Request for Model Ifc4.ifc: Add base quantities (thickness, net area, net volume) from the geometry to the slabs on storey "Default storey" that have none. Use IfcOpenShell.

First a look at what the model holds.

```python
import ifcopenshell
import ifcopenshell.util.element
import ifcopenshell.util.unit

model = ifcopenshell.open("Model Ifc4.ifc")
print(model.schema)
for unit_type in ("LENGTHUNIT", "AREAUNIT", "VOLUMEUNIT"):
    print(unit_type, ifcopenshell.util.unit.calculate_unit_scale(model, unit_type))
storey = next(s for s in model.by_type("IfcBuildingStorey") if s.Name == "Default storey")
slabs = [e for e in ifcopenshell.util.element.get_decomposition(storey) if e.is_a("IfcSlab")]
for e in sorted(slabs, key=lambda e: e.id()):
    print(e.id(), e.is_a(), e.Name, list(ifcopenshell.util.element.get_psets(e, qtos_only=True)), sep=" | ")
```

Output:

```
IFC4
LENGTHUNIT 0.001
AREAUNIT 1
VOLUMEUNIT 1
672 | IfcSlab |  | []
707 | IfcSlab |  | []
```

```python
import ifcopenshell
import ifcopenshell.api.pset
import ifcopenshell.geom
import ifcopenshell.util.element
import ifcopenshell.util.shape
import ifcopenshell.util.unit

model = ifcopenshell.open("Model Ifc4.ifc")
unit_scale = ifcopenshell.util.unit.calculate_unit_scale(model)
area_scale = ifcopenshell.util.unit.calculate_unit_scale(model, "AREAUNIT")
volume_scale = ifcopenshell.util.unit.calculate_unit_scale(model, "VOLUMEUNIT")
settings = ifcopenshell.geom.settings()

storey = next(s for s in model.by_type("IfcBuildingStorey") if s.Name == "Default storey")
slabs = [e for e in ifcopenshell.util.element.get_decomposition(storey) if e.is_a("IfcSlab")]

for e in sorted(slabs, key=lambda e: e.id()):
    if ifcopenshell.util.element.get_psets(e, qtos_only=True, should_inherit=False):
        continue
    # Geometry comes back in metres, in the element's own axes.
    shape = ifcopenshell.geom.create_shape(settings, e)
    values = {
        "Width": ifcopenshell.util.shape.get_z(shape.geometry) / unit_scale,
        "NetArea": ifcopenshell.util.shape.get_footprint_area(shape.geometry) / area_scale,
        "NetVolume": ifcopenshell.util.shape.get_volume(shape.geometry) / volume_scale,
    }
    qto = ifcopenshell.api.pset.add_qto(model, product=e, name="Qto_SlabBaseQuantities")
    ifcopenshell.api.pset.edit_qto(model, qto=qto, properties=values)
    print(e.id(), {k: round(v, 3) for k, v in values.items()})

model.write("Model Ifc4_v2.ifc")
```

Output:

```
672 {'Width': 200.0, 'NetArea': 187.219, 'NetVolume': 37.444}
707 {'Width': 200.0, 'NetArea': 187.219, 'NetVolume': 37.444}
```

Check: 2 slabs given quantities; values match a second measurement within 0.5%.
